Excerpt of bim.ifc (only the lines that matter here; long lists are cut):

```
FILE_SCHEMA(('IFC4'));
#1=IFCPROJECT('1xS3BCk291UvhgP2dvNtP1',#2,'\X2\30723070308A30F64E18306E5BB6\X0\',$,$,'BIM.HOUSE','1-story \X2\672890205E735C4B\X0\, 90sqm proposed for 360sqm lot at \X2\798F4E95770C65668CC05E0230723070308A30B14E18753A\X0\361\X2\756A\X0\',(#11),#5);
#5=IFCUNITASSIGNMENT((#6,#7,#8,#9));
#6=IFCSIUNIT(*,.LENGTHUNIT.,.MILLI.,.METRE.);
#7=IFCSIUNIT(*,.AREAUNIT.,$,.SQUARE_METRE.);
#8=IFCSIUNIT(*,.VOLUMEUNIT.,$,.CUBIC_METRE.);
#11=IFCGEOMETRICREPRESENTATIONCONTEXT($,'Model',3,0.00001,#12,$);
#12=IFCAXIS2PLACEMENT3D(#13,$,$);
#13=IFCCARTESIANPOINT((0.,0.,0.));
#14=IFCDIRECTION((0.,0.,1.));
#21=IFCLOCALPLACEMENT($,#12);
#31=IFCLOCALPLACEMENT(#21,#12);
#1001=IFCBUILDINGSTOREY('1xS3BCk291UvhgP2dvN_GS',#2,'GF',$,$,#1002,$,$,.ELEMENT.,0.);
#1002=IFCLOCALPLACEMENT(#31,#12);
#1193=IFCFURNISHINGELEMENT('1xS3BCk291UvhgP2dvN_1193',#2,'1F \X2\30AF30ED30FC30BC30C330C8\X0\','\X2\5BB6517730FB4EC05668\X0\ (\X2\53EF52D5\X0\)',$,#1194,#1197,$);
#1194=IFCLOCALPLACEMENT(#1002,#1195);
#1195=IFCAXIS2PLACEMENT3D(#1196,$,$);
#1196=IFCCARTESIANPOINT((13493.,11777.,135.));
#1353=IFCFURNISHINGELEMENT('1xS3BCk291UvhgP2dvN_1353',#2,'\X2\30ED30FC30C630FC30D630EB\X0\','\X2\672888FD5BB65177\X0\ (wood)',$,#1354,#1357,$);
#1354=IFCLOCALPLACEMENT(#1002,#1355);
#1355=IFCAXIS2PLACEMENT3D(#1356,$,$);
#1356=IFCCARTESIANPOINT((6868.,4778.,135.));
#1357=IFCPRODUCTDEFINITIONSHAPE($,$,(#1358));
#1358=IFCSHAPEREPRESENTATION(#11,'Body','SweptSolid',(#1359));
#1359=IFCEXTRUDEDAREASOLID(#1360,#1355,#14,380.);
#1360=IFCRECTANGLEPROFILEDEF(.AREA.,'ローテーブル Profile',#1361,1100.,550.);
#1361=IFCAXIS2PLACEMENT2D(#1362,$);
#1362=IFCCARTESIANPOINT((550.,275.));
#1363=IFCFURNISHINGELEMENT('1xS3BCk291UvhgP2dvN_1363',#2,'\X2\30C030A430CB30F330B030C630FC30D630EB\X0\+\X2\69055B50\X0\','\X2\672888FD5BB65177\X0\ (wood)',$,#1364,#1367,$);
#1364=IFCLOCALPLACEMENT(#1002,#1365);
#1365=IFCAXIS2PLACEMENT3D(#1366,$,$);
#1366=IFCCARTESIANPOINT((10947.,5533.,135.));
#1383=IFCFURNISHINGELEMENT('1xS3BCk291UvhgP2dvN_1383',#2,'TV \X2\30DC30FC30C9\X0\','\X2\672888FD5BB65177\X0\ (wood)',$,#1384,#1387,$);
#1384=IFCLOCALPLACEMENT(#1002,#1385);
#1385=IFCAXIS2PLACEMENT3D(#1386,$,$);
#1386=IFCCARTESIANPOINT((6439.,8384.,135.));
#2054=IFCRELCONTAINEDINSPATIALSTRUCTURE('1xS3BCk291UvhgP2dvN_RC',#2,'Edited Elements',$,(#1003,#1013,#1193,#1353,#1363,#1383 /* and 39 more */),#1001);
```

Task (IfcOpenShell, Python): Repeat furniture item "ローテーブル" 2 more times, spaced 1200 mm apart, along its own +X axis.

```python
import ifcopenshell
import ifcopenshell.api.geometry
import ifcopenshell.api.root
import ifcopenshell.util.element
import ifcopenshell.util.placement

model = ifcopenshell.open("bim.ifc")


def reuse_history(source, copy):
    """copy_class also copies each property set's owner history, people and application; keep the originals."""
    for rel in copy.IsDefinedBy:
        if rel.is_a("IfcRelDefinesByProperties") and (history := rel.RelatingPropertyDefinition.OwnerHistory):
            rel.RelatingPropertyDefinition.OwnerHistory = source.OwnerHistory
            ifcopenshell.util.element.remove_deep2(model, history)


source = model.by_guid("1xS3BCk291UvhgP2dvN_1353")
base = ifcopenshell.util.placement.get_local_placement(source.ObjectPlacement)
step = base[:3, 0] * 1200.0

for i in range(1, 3):
    copy = ifcopenshell.api.root.copy_class(model, product=source)
    copy.Representation = ifcopenshell.util.element.copy_deep(
        model, source.Representation, exclude=["IfcGeometricRepresentationContext", "IfcRepresentationMap"]
    )
    reuse_history(source, copy)
    matrix = base.copy()
    matrix[:3, 3] += i * step
    print("added at", matrix[:3, 3].round(3) + 0.0)
    ifcopenshell.api.geometry.edit_object_placement(model, product=copy, matrix=matrix, is_si=False)

model.write("bim_v2.ifc")
```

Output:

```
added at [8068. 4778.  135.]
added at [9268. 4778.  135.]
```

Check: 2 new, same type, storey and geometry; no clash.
